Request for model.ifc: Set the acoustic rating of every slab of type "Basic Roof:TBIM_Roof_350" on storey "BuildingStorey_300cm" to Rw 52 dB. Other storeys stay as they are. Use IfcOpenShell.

First a look at what the model holds.

```python
import ifcopenshell
import ifcopenshell.util.element

model = ifcopenshell.open("model.ifc")
print(model.schema)
storey = next(s for s in model.by_type("IfcBuildingStorey") if s.Name == "BuildingStorey_300cm")
slabs = [e for e in ifcopenshell.util.element.get_decomposition(storey) if e.is_a("IfcSlab")]
seen = {}
for e in slabs:
    element_type = ifcopenshell.util.element.get_type(e)
    key = (element_type.Name if element_type != e and element_type else None, ifcopenshell.util.element.get_pset(e, "Pset_SlabCommon", "AcousticRating"))
    seen[key] = seen.get(key, 0) + 1
for (name, value), count in sorted(seen.items(), key=str):
    print(count, "x", name, "|", value)
```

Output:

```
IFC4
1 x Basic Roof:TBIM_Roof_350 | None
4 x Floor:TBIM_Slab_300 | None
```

```python
import ifcopenshell
import ifcopenshell.api.pset
import ifcopenshell.util.element

model = ifcopenshell.open("model.ifc")

storey = next(s for s in model.by_type("IfcBuildingStorey") if s.Name == "BuildingStorey_300cm")
slabs = [e for e in ifcopenshell.util.element.get_decomposition(storey) if e.is_a("IfcSlab")]

count = 0
for e in slabs:
    element_type = ifcopenshell.util.element.get_type(e)
    if element_type in (None, e) or element_type.Name != "Basic Roof:TBIM_Roof_350":
        continue
    # add_pset returns the element's existing set when there is one.
    pset = ifcopenshell.api.pset.add_pset(model, product=e, name="Pset_SlabCommon")
    ifcopenshell.api.pset.edit_pset(model, pset=pset, properties={"AcousticRating": "Rw 52 dB"})
    count += 1

print(count, "slabs updated")

model.write("model_edited.ifc")
```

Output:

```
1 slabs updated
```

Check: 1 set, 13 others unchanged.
